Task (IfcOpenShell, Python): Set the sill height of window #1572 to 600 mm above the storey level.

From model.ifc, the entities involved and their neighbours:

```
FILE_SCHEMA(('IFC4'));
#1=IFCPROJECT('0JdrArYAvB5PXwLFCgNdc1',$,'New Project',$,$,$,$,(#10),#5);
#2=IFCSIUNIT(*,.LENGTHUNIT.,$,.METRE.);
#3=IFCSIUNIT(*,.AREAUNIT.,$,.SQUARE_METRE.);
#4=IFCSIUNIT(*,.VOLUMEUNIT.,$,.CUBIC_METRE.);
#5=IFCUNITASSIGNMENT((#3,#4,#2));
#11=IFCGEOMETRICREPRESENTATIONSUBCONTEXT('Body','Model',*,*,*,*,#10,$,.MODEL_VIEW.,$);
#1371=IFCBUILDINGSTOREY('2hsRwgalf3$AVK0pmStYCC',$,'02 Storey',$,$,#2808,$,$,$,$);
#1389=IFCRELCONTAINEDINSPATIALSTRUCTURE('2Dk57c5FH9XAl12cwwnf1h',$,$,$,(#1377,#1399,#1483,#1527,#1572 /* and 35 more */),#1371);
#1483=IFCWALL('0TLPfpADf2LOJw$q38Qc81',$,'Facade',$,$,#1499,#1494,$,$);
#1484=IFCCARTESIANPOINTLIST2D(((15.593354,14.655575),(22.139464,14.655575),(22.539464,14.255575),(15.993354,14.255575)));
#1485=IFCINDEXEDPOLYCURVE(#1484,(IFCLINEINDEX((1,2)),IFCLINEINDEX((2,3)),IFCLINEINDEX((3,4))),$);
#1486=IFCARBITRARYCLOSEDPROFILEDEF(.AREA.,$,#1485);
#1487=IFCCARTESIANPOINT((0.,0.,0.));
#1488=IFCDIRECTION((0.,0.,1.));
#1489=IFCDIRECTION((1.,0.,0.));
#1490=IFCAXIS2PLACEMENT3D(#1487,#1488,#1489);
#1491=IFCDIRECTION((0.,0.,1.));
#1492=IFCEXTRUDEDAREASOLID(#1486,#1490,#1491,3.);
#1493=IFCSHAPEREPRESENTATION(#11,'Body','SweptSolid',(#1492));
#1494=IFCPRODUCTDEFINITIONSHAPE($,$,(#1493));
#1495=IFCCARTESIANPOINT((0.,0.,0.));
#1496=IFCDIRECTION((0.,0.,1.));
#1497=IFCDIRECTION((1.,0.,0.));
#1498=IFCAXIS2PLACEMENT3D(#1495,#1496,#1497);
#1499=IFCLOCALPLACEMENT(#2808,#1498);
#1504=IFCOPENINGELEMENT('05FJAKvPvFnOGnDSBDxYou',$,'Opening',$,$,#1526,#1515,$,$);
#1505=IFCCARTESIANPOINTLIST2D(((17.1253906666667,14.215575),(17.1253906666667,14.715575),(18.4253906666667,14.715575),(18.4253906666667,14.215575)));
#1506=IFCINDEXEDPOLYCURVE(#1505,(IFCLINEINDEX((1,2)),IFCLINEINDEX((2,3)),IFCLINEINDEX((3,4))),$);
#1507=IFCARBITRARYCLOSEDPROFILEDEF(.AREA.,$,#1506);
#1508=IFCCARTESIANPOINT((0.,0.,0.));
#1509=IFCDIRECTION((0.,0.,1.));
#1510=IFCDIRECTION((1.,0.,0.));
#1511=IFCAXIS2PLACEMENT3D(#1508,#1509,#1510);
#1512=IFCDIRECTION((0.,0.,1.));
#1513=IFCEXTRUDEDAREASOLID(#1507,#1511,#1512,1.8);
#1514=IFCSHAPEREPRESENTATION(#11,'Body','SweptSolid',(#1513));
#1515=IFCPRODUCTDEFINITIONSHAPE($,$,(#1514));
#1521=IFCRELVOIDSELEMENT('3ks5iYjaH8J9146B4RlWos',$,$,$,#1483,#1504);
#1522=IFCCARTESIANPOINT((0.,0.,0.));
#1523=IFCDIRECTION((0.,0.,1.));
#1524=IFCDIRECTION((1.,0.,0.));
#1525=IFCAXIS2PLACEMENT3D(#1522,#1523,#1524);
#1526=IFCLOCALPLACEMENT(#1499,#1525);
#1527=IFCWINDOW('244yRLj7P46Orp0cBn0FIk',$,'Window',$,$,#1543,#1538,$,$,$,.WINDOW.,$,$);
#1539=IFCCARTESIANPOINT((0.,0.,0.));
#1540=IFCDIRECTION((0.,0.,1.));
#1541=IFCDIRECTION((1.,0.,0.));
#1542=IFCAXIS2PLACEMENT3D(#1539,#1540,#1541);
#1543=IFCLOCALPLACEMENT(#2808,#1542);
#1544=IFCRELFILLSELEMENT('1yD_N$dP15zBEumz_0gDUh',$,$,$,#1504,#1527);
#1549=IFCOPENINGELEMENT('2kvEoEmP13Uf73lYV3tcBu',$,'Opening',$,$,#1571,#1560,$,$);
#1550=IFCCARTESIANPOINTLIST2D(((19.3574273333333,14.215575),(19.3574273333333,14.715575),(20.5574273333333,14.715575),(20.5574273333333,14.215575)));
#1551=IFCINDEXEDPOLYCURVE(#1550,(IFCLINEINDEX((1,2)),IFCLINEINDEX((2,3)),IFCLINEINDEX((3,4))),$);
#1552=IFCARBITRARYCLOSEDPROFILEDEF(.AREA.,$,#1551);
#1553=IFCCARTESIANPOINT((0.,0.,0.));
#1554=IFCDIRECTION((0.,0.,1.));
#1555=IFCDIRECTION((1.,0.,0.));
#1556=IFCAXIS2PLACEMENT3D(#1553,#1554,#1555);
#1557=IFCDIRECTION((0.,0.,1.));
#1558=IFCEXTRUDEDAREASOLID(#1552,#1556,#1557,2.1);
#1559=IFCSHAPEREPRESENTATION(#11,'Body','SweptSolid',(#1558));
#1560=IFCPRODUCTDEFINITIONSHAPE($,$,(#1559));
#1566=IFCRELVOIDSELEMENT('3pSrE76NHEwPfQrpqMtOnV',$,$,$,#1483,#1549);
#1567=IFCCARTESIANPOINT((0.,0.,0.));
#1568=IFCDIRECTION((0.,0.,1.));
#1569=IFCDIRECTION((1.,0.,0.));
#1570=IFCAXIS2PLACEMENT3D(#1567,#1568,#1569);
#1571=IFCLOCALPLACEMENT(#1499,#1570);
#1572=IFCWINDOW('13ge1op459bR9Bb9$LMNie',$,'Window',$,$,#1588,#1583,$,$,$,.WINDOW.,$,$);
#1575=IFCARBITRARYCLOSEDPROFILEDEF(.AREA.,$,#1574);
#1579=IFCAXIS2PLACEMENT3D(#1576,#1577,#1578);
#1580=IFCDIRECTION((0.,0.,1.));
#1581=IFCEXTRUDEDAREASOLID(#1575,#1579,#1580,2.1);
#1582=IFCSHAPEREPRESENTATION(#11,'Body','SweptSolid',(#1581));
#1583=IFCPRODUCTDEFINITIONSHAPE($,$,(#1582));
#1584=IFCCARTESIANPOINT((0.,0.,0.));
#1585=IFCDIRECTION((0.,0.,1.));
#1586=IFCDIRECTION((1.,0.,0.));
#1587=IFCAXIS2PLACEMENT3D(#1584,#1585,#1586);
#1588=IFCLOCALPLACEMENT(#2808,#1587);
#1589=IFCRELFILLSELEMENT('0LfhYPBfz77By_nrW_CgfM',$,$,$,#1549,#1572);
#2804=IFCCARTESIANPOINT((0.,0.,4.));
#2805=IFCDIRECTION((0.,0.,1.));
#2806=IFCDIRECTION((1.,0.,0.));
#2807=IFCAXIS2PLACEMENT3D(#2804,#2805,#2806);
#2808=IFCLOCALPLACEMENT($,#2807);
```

```python
import numpy as np
import ifcopenshell
import ifcopenshell.api.geometry
import ifcopenshell.geom
import ifcopenshell.util.element
import ifcopenshell.util.placement
import ifcopenshell.util.shape
import ifcopenshell.util.unit

model = ifcopenshell.open("model.ifc")
unit_scale = ifcopenshell.util.unit.calculate_unit_scale(model)

window = model.by_guid("13ge1op459bR9Bb9$LMNie")
opening = window.FillsVoids[0].RelatingOpeningElement
storey = ifcopenshell.util.element.get_container(window, ifc_class="IfcBuildingStorey")
level = ifcopenshell.util.placement.get_local_placement(storey.ObjectPlacement)[2, 3]

# The opening's origin need not be at the sill, so measure its lowest point.
shape = ifcopenshell.geom.create_shape(ifcopenshell.geom.settings(), opening)
bottom = ifcopenshell.util.shape.get_shape_bottom_elevation(shape, shape.geometry) / unit_scale
dz = level + 0.6 - bottom

shift = np.array([0.0, 0.0, dz])
# The window is not placed relative to its opening, so move both.
for product in (opening, window):
    matrix = ifcopenshell.util.placement.get_local_placement(product.ObjectPlacement)
    matrix[:3, 3] += shift
    ifcopenshell.api.geometry.edit_object_placement(model, product=product, matrix=matrix, is_si=False)

print(f"moved by {dz * unit_scale:+.3f} m")

model.write("model_updated.ifc")
```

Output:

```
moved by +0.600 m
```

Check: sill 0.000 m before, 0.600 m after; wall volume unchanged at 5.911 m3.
